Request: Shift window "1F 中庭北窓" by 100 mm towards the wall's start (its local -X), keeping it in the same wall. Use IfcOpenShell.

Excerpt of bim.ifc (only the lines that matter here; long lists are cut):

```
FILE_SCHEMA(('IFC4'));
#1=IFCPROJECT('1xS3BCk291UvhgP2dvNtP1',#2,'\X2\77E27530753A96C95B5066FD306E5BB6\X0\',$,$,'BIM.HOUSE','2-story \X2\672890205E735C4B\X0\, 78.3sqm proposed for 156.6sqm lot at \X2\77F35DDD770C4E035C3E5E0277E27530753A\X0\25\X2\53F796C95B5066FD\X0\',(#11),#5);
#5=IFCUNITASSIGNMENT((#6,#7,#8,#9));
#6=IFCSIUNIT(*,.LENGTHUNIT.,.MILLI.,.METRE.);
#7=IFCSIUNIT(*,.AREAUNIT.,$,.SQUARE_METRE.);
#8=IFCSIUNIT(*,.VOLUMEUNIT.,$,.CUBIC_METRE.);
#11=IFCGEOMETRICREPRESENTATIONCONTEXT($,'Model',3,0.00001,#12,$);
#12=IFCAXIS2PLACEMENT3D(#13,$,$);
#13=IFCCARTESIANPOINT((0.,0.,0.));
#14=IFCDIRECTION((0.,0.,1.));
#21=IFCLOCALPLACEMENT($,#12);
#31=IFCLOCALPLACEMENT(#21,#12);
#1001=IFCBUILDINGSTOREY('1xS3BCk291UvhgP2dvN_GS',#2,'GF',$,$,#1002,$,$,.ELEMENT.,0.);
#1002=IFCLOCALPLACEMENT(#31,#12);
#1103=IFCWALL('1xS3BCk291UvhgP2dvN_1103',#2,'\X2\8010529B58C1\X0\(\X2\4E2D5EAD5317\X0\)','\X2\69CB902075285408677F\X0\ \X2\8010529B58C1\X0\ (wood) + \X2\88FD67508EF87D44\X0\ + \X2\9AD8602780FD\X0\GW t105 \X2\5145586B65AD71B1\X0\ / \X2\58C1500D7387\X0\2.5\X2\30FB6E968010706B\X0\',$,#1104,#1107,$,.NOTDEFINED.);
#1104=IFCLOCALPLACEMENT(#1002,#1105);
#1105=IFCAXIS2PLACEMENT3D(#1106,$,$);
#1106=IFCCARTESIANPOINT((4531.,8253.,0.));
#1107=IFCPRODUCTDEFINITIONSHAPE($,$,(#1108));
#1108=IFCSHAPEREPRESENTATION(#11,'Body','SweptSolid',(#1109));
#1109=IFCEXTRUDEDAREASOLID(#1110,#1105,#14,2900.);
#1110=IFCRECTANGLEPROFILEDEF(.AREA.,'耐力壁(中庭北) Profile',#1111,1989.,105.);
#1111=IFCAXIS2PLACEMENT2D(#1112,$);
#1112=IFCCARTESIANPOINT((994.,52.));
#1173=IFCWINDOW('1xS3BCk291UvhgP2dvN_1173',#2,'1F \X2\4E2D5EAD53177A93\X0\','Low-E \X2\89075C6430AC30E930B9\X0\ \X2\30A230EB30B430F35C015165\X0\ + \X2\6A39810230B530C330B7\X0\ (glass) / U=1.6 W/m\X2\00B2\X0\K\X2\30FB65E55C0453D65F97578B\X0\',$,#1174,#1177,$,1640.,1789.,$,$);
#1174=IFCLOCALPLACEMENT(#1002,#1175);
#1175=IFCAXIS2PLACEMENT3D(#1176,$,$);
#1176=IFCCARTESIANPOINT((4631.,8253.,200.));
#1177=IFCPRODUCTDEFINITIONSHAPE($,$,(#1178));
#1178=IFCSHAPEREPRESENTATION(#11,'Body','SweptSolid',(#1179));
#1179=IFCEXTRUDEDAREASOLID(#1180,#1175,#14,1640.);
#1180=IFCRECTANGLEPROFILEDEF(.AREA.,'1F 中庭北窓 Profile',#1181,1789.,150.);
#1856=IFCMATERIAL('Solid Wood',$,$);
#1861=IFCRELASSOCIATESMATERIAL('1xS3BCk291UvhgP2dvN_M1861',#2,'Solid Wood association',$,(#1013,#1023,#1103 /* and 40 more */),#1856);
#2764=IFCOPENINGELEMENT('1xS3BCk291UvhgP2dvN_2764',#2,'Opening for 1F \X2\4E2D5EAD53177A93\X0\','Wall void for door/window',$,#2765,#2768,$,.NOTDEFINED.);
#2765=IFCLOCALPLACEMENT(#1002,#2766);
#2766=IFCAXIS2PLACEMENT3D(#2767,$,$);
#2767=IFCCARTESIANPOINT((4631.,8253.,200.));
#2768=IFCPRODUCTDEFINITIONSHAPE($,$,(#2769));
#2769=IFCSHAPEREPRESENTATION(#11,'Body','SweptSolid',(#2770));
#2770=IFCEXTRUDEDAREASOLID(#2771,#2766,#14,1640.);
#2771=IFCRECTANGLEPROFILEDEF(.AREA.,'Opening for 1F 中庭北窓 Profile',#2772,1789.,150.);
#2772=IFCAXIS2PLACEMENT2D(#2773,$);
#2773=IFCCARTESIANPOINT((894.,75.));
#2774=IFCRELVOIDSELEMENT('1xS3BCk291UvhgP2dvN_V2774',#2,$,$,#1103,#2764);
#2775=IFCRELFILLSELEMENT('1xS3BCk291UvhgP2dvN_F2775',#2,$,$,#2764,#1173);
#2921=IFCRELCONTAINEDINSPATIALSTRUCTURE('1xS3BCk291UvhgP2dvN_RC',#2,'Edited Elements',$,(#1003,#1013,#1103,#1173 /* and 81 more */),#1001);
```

```python
import ifcopenshell
import ifcopenshell.api.geometry
import ifcopenshell.util.placement
import ifcopenshell.util.unit

model = ifcopenshell.open("bim.ifc")
unit_scale = ifcopenshell.util.unit.calculate_unit_scale(model)

window = model.by_guid("1xS3BCk291UvhgP2dvN_1173")
opening = window.FillsVoids[0].RelatingOpeningElement
wall = opening.VoidsElements[0].RelatingBuildingElement

wall_matrix = ifcopenshell.util.placement.get_local_placement(wall.ObjectPlacement)
shift = wall_matrix[:3, 0] * -0.1 / unit_scale
before = ifcopenshell.util.placement.get_local_placement(window.ObjectPlacement)[:3, 3].copy()

# The window is not placed relative to its opening, so move both.
for product in (opening, window):
    matrix = ifcopenshell.util.placement.get_local_placement(product.ObjectPlacement)
    matrix[:3, 3] += shift
    ifcopenshell.api.geometry.edit_object_placement(model, product=product, matrix=matrix, is_si=False)

after = ifcopenshell.util.placement.get_local_placement(window.ObjectPlacement)[:3, 3]
print("window moved by", (after - before).round(3) + 0.0)

model.write("bim_rev.ifc")
```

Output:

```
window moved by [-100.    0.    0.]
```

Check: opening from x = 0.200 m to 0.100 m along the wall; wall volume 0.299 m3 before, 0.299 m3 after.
